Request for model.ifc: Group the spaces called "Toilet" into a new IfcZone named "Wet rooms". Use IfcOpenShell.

First a look at what the model holds.

```python
import ifcopenshell

model = ifcopenshell.open("model.ifc")
print(model.schema)
seen = {}
for space in model.by_type("IfcSpace"):
    seen[space.LongName] = seen.get(space.LongName, 0) + 1
for name, count in sorted(seen.items(), key=str):
    print(count, "x", name)
print("zones:", [z.Name for z in model.by_type("IfcZone")][:20])
```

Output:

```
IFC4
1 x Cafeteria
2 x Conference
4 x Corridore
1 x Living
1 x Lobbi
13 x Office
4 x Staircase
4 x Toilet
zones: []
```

```python
import ifcopenshell
import ifcopenshell.api.group
import ifcopenshell.api.root

model = ifcopenshell.open("model.ifc")

names = {"Toilet"}
spaces = [s for s in model.by_type("IfcSpace") if s.LongName in names]

zone = ifcopenshell.api.root.create_entity(model, ifc_class="IfcZone", name="Wet rooms")
ifcopenshell.api.group.assign_group(model, products=spaces, group=zone)
print(len(spaces), "spaces in", zone.Name)

model.write("model_v2.ifc")
```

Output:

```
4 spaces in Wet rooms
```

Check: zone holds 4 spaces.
